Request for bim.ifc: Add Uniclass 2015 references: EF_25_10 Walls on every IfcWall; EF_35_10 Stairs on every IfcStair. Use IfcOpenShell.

First a look at what the model holds.

```python
import ifcopenshell

model = ifcopenshell.open("bim.ifc")
print(model.schema)
print("classifications:", [c.Name for c in model.by_type("IfcClassification")])
for ifc_class in ("IfcDoor", "IfcRoof", "IfcStair", "IfcWall", "IfcWindow"):
    print(ifc_class, len(model.by_type(ifc_class)))
```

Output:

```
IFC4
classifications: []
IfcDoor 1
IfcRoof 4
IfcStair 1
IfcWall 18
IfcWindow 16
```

```python
import ifcopenshell
import ifcopenshell.api.classification

model = ifcopenshell.open("bim.ifc")

system = ifcopenshell.api.classification.add_classification(model, classification="Uniclass 2015")

codes = {
    "IfcWall": ("EF_25_10", "Walls"),
    "IfcStair": ("EF_35_10", "Stairs"),
}
for ifc_class, (code, name) in codes.items():
    products = model.by_type(ifc_class)
    ifcopenshell.api.classification.add_reference(
        model, products=products, classification=system, identification=code, name=name
    )
    print(code, len(products))

model.write("bim_updated.ifc")
```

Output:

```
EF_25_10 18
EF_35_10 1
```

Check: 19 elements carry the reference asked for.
